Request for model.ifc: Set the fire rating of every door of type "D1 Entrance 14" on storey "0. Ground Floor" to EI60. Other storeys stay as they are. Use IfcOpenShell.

First a look at what the model holds.

```python
import ifcopenshell
import ifcopenshell.util.element

model = ifcopenshell.open("model.ifc")
print(model.schema)
storey = next(s for s in model.by_type("IfcBuildingStorey") if s.Name == "0. Ground Floor")
doors = [e for e in ifcopenshell.util.element.get_decomposition(storey) if e.is_a("IfcDoor")]
seen = {}
for e in doors:
    element_type = ifcopenshell.util.element.get_type(e)
    key = (element_type.Name if element_type != e and element_type else None, ifcopenshell.util.element.get_pset(e, "Pset_DoorCommon", "FireRating"))
    seen[key] = seen.get(key, 0) + 1
for (name, value), count in sorted(seen.items(), key=str):
    print(count, "x", name, "|", value)
```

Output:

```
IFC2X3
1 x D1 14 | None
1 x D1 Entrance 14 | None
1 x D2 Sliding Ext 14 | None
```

```python
import ifcopenshell
import ifcopenshell.api.pset
import ifcopenshell.util.element

model = ifcopenshell.open("model.ifc")

storey = next(s for s in model.by_type("IfcBuildingStorey") if s.Name == "0. Ground Floor")
doors = [e for e in ifcopenshell.util.element.get_decomposition(storey) if e.is_a("IfcDoor")]

count = 0
for e in doors:
    element_type = ifcopenshell.util.element.get_type(e)
    if element_type in (None, e) or element_type.Name != "D1 Entrance 14":
        continue
    # add_pset returns the element's existing set when there is one.
    pset = ifcopenshell.api.pset.add_pset(model, product=e, name="Pset_DoorCommon")
    ifcopenshell.api.pset.edit_pset(model, pset=pset, properties={"FireRating": "EI60"})
    count += 1

print(count, "doors updated")

model.write("model-out.ifc")
```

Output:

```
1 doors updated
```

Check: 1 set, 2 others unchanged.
